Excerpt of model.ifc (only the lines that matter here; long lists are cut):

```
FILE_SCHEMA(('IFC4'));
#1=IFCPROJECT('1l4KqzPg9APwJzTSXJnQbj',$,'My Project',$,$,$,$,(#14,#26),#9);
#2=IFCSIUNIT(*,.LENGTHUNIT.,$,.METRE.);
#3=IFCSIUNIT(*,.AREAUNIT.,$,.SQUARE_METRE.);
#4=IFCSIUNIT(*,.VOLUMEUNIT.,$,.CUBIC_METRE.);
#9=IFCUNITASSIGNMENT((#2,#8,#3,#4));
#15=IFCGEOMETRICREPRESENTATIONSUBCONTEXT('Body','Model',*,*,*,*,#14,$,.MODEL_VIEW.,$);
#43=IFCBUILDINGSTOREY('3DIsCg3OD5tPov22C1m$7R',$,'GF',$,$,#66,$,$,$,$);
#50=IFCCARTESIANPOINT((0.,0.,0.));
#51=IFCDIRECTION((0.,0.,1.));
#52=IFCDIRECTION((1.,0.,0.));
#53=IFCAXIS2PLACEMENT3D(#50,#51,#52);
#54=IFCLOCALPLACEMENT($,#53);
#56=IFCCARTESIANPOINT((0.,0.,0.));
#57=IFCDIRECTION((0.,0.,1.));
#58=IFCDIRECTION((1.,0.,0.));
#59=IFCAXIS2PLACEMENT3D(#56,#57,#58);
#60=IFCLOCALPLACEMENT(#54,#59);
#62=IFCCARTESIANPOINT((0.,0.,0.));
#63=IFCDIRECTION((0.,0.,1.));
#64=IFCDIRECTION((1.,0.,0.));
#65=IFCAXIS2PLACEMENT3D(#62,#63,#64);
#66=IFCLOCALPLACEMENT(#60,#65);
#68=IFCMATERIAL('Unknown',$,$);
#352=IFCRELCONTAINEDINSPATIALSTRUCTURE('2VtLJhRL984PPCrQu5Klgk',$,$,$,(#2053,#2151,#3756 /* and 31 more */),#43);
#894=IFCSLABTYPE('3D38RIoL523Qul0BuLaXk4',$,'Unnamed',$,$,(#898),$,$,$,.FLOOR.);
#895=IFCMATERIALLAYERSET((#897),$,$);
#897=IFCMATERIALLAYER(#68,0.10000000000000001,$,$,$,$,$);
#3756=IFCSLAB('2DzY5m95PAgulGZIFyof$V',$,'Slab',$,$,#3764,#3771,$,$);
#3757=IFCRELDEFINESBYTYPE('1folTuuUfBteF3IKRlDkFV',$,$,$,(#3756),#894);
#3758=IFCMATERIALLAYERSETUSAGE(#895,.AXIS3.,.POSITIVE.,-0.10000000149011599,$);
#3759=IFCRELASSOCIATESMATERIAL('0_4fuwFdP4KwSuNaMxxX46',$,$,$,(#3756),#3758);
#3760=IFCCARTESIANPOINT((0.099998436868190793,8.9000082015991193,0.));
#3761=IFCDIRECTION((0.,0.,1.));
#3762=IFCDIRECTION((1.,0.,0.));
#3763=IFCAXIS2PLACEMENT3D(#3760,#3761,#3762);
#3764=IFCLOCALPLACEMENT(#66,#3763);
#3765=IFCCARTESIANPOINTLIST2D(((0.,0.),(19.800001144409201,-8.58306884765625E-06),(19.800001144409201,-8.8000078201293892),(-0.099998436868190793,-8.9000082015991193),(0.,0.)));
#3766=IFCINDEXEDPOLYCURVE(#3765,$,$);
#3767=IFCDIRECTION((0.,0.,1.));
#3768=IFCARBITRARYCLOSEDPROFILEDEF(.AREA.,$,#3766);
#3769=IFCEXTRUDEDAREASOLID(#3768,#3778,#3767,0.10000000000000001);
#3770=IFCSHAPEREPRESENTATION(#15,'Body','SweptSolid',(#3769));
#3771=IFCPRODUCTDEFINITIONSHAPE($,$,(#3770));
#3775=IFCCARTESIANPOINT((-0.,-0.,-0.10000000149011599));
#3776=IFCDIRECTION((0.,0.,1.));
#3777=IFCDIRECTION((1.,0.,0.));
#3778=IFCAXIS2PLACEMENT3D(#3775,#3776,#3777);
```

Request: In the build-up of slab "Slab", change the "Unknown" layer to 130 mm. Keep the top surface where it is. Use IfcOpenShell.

```python
import ifcopenshell
import ifcopenshell.util.element
import ifcopenshell.util.representation

model = ifcopenshell.open("model.ifc")

layer_set = model.by_id(895)
layer = next(l for l in layer_set.MaterialLayers if l.Material and l.Material.Name == "Unknown")
change = 0.13 - layer.LayerThickness
layer.LayerThickness += change

# Geometry does not follow the layer set by itself.
slabs = [e for e in ifcopenshell.util.element.get_elements_by_material(model, layer_set) if e.is_a("IfcSlab")]
for slab in sorted(slabs, key=lambda e: e.id()):
    body = ifcopenshell.util.representation.get_representation(slab, "Model", "Body")
    solid = body.Items[0]
    old_depth = solid.Depth
    solid.Depth += change
    # Extruded upwards: lower the start of the extrusion so the top stays.
    x, y, z = solid.Position.Location.Coordinates
    solid.Position.Location = model.createIfcCartesianPoint((x, y, z - change))
    print(slab.id(), f"{old_depth:g} -> {solid.Depth:g}")

# The layers are counted up from the underside, which has moved.
for usage in {ifcopenshell.util.element.get_material(slab) for slab in slabs}:
    usage.OffsetFromReferenceLine -= change

model.write("model_updated.ifc")
```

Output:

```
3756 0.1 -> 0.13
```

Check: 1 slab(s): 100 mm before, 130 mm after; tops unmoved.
